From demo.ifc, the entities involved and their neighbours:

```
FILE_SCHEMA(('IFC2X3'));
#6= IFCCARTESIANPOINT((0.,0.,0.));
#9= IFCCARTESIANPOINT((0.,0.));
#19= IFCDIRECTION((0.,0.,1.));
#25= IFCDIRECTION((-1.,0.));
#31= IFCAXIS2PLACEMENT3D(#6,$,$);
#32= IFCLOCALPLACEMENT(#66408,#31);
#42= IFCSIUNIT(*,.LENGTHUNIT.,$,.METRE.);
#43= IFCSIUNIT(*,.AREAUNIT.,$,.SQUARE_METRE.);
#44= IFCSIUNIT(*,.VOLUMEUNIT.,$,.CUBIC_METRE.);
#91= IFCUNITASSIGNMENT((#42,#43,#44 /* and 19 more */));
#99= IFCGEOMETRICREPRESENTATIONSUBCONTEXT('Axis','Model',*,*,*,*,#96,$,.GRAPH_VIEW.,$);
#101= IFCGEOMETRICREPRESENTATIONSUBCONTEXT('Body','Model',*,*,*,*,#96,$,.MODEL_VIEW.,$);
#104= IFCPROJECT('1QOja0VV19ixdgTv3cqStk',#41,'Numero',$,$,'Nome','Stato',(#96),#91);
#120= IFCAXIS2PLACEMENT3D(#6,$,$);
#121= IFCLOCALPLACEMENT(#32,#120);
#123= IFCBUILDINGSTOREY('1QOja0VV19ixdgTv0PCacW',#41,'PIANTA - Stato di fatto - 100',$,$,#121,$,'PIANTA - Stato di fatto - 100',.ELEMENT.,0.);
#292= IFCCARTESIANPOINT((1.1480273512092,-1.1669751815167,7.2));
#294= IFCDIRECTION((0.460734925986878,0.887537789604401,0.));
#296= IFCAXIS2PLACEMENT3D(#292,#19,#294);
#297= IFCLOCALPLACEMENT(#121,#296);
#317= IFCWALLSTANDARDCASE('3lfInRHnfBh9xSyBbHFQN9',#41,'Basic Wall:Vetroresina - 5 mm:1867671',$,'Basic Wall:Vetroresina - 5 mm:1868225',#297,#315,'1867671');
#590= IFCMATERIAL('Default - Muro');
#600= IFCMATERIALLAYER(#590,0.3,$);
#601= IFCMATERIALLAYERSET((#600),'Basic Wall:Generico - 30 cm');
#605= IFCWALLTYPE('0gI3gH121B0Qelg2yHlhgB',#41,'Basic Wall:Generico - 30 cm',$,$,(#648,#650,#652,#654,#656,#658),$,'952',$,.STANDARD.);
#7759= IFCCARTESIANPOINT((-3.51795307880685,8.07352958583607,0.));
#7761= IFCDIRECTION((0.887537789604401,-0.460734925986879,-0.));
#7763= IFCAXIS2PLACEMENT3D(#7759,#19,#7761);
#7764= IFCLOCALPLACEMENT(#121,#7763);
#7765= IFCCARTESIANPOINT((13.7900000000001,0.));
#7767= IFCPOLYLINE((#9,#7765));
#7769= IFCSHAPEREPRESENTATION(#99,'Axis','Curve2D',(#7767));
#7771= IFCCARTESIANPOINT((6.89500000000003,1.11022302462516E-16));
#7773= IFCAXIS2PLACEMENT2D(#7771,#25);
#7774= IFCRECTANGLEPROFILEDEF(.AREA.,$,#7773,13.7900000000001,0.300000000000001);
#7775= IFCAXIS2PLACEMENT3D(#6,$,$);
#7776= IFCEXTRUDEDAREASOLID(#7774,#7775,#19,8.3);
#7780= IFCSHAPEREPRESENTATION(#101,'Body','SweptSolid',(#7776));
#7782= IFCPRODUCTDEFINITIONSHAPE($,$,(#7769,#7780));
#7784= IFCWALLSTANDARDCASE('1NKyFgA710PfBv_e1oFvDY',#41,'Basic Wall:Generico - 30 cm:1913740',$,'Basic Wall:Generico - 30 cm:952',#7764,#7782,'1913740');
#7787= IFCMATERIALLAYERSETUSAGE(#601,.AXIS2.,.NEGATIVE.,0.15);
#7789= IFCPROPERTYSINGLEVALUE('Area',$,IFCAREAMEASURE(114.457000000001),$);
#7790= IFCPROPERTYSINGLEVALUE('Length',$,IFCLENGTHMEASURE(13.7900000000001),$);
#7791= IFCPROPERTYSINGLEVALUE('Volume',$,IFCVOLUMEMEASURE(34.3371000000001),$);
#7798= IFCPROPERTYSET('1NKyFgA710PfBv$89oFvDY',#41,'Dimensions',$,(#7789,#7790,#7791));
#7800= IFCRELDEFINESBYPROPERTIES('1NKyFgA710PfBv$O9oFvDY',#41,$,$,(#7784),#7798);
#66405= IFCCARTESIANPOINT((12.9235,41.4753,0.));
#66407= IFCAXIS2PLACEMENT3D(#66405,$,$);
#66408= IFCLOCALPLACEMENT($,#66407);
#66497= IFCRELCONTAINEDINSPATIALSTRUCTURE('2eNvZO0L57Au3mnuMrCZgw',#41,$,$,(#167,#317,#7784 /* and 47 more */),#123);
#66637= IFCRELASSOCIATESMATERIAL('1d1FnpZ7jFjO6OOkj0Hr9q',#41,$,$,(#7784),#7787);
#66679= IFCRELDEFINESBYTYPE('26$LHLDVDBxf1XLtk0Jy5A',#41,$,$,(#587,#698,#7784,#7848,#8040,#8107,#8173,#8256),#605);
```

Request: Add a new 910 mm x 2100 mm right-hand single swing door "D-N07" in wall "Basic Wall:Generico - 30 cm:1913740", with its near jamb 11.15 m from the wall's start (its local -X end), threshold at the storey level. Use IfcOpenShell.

```python
import numpy as np
import ifcopenshell
import ifcopenshell.api.feature
import ifcopenshell.api.geometry
import ifcopenshell.api.pset
import ifcopenshell.api.root
import ifcopenshell.api.spatial
import ifcopenshell.api.type
import ifcopenshell.geom
import ifcopenshell.util.element
import ifcopenshell.util.placement
import ifcopenshell.util.representation
import ifcopenshell.util.shape
import ifcopenshell.util.unit

model = ifcopenshell.open("demo.ifc")
unit_scale = ifcopenshell.util.unit.calculate_unit_scale(model)
area_scale = ifcopenshell.util.unit.calculate_unit_scale(model, "AREAUNIT")
volume_scale = ifcopenshell.util.unit.calculate_unit_scale(model, "VOLUMEUNIT")
settings = ifcopenshell.geom.settings()


def volume(element):
    """Net volume in cubic metres, openings subtracted."""
    shape = ifcopenshell.geom.create_shape(settings, element)
    return ifcopenshell.util.shape.get_volume(shape.geometry)


wall = model.by_guid("1NKyFgA710PfBv_e1oFvDY")
storey = ifcopenshell.util.element.get_container(wall, ifc_class="IfcBuildingStorey")
context = ifcopenshell.util.representation.get_context(model, "Model", "Body", "MODEL_VIEW")
before = volume(wall)

width, height, from_end, sill = 0.91, 2.1, 11.15, 0.0  # metres

# The wall runs along its own X axis, and the end named is its -X end.
wall_shape = ifcopenshell.geom.create_shape(settings, wall)
x, y, z = ifcopenshell.util.shape.get_vertices(wall_shape.geometry).T
start = x.min() + from_end
face, thickness = float(y.min()), float(y.max() - y.min())
wall_matrix = ifcopenshell.util.placement.get_local_placement(wall.ObjectPlacement)
level = ifcopenshell.util.placement.get_local_placement(storey.ObjectPlacement)[2, 3]


def in_wall(x, y):
    """Placement at x, y metres in the wall's axes, at sill height."""
    matrix = wall_matrix.copy()
    matrix[:, 3] = wall_matrix @ np.array([x / unit_scale, y / unit_scale, 0.0, 1.0])
    matrix[2, 3] = level + sill / unit_scale
    return matrix


# Opening: a box that overshoots both wall faces by 50 mm.
opening = ifcopenshell.api.root.create_entity(model, ifc_class="IfcOpeningElement")
box = ifcopenshell.api.geometry.add_wall_representation(
    model, context=context, length=width, height=height, thickness=thickness + 0.1
)
ifcopenshell.api.geometry.assign_representation(model, product=opening, representation=box)
ifcopenshell.api.geometry.edit_object_placement(model, product=opening, matrix=in_wall(start, face - 0.05), is_si=False)
ifcopenshell.api.feature.add_feature(model, feature=opening, element=wall)

door = ifcopenshell.api.root.create_entity(model, ifc_class="IfcDoor", name="D-N07")
door.OverallWidth, door.OverallHeight = width / unit_scale, height / unit_scale
body = ifcopenshell.api.geometry.add_door_representation(
    model,
    context=context,
    overall_width=door.OverallWidth,
    overall_height=door.OverallHeight,
    operation_type="SINGLE_SWING_RIGHT",
    lining_properties={"LiningDepth": thickness / unit_scale, "ThresholdDepth": thickness / unit_scale},
)
ifcopenshell.api.geometry.assign_representation(model, product=door, representation=body)
ifcopenshell.api.spatial.assign_container(model, products=[door], relating_structure=storey)
fills = ifcopenshell.api.feature.add_filling(model, opening=opening, element=door)
fills.OwnerHistory = door.OwnerHistory  # required in IFC2X3

# IFC2X3 keeps the operation on the door style.
style = ifcopenshell.api.root.create_entity(model, ifc_class="IfcDoorStyle", name="D-N07")
style.OperationType, style.ConstructionType = "SINGLE_SWING_RIGHT", "NOTDEFINED"
style.ParameterTakesPrecedence = style.Sizeable = False
ifcopenshell.api.type.assign_type(model, related_objects=[door], relating_type=style)

# The lining spans the wall, so the door starts at the wall face.
ifcopenshell.api.geometry.edit_object_placement(model, product=door, matrix=in_wall(start, face), is_si=False)

after = volume(wall)

# Update the wall's stored quantities.
pset = model.by_id(ifcopenshell.util.element.get_pset(wall, "Dimensions", should_inherit=False)["id"])
ifcopenshell.api.pset.edit_pset(model, pset=pset, properties={
    "Area": model.create_entity("IfcAreaMeasure", after / thickness / area_scale),
    "Volume": model.create_entity("IfcVolumeMeasure", after / volume_scale),
})

print(f"wall volume {before:.3f} -> {after:.3f} m3")

model.write("demo_updated.ifc")
```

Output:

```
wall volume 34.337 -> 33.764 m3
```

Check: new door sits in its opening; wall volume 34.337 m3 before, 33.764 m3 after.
